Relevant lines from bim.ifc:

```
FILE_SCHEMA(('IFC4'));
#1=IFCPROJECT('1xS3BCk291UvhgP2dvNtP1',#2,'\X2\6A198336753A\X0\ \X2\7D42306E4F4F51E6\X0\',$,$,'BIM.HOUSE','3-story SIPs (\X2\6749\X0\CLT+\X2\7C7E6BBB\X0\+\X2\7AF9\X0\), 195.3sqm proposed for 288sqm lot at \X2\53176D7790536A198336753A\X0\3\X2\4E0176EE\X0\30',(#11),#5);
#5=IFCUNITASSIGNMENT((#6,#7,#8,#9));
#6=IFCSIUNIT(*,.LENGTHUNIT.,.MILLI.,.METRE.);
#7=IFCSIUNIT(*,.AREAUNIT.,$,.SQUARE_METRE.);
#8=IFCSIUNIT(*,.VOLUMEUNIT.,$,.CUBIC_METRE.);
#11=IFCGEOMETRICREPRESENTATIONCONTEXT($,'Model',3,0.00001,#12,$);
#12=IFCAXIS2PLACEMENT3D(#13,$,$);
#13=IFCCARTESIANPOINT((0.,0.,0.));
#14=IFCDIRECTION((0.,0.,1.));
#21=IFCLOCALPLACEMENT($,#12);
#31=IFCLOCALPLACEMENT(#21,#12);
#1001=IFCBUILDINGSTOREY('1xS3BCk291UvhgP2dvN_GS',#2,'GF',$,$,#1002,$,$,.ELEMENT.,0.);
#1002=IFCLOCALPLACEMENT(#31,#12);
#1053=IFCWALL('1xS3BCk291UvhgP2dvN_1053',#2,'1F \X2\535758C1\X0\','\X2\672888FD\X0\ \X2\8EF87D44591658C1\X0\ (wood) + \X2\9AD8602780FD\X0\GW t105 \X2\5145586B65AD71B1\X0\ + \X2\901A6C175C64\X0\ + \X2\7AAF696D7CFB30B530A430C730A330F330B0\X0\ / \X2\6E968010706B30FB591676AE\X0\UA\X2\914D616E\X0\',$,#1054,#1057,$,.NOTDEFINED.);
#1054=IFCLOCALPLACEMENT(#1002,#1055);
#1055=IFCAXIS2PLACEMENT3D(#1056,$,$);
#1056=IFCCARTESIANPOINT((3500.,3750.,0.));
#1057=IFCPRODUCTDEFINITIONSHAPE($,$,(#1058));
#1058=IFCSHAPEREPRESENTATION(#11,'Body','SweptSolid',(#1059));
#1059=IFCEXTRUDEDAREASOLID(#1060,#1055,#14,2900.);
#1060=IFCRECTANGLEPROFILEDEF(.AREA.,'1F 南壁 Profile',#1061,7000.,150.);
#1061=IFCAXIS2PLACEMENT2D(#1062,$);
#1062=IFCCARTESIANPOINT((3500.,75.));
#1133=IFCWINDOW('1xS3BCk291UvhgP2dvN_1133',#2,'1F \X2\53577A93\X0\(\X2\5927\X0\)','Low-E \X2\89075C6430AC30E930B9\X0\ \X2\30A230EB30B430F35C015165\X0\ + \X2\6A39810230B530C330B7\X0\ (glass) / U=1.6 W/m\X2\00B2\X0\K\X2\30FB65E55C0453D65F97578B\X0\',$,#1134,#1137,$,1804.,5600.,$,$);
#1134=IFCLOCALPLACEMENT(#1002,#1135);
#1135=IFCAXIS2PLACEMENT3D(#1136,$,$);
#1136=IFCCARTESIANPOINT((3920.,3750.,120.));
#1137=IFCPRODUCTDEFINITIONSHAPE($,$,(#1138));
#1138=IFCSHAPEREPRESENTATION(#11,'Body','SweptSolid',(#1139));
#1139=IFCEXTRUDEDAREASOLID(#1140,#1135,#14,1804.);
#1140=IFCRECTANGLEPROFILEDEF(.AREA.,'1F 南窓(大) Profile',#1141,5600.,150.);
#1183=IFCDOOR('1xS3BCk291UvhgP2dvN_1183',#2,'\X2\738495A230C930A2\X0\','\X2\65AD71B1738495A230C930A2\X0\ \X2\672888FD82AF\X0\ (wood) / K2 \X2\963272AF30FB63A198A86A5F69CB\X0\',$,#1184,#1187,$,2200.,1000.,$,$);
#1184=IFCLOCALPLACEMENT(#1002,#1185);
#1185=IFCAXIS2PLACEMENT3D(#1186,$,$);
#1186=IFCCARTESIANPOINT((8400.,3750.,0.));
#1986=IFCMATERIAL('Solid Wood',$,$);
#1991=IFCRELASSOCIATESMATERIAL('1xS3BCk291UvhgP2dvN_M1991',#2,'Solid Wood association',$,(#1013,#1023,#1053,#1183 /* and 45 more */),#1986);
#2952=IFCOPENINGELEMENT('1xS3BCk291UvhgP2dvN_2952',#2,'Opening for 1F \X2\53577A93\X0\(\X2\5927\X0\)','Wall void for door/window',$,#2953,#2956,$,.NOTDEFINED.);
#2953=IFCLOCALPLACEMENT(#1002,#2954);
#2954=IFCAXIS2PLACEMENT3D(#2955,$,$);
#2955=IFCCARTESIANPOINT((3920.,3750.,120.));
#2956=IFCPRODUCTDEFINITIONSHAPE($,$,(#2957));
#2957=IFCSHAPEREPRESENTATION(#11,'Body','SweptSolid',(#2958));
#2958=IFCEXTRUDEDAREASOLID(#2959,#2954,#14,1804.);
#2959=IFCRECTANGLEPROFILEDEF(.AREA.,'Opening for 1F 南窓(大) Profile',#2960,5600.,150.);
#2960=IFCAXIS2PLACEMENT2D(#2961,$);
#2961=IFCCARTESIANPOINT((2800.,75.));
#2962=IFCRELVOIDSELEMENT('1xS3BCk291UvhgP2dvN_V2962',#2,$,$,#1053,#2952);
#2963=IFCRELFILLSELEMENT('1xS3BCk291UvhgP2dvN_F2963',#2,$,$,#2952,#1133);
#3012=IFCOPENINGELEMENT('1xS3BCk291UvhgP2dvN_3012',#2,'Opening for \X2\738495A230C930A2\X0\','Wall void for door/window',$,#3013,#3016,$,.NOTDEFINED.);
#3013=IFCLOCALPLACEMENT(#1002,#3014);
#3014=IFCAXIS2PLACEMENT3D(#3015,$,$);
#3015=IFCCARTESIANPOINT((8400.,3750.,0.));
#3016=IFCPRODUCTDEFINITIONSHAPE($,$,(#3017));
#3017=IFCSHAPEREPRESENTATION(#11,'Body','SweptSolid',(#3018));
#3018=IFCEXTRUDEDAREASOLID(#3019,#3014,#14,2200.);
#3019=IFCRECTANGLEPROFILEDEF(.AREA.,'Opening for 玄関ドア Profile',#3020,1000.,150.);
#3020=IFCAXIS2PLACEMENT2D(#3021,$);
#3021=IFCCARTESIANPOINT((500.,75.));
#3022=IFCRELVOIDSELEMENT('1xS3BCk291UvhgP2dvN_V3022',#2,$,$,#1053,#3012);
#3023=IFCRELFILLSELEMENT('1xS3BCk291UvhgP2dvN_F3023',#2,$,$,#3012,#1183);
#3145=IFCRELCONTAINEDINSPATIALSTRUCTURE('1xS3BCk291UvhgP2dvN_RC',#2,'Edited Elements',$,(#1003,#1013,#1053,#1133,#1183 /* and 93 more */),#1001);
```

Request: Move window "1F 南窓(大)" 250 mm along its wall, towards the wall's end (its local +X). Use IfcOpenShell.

```python
import ifcopenshell
import ifcopenshell.api.geometry
import ifcopenshell.util.placement
import ifcopenshell.util.unit

model = ifcopenshell.open("bim.ifc")
unit_scale = ifcopenshell.util.unit.calculate_unit_scale(model)

window = model.by_id(1133)
opening = window.FillsVoids[0].RelatingOpeningElement
wall = opening.VoidsElements[0].RelatingBuildingElement

wall_matrix = ifcopenshell.util.placement.get_local_placement(wall.ObjectPlacement)
shift = wall_matrix[:3, 0] * 0.25 / unit_scale
before = ifcopenshell.util.placement.get_local_placement(window.ObjectPlacement)[:3, 3].copy()

# The window is not placed relative to its opening, so move both.
for product in (opening, window):
    matrix = ifcopenshell.util.placement.get_local_placement(product.ObjectPlacement)
    matrix[:3, 3] += shift
    ifcopenshell.api.geometry.edit_object_placement(model, product=product, matrix=matrix, is_si=False)

after = ifcopenshell.util.placement.get_local_placement(window.ObjectPlacement)[:3, 3]
print("window moved by", (after - before).round(3) + 0.0)

model.write("bim-out.ifc")
```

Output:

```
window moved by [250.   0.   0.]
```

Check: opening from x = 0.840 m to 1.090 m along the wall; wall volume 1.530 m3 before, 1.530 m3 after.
